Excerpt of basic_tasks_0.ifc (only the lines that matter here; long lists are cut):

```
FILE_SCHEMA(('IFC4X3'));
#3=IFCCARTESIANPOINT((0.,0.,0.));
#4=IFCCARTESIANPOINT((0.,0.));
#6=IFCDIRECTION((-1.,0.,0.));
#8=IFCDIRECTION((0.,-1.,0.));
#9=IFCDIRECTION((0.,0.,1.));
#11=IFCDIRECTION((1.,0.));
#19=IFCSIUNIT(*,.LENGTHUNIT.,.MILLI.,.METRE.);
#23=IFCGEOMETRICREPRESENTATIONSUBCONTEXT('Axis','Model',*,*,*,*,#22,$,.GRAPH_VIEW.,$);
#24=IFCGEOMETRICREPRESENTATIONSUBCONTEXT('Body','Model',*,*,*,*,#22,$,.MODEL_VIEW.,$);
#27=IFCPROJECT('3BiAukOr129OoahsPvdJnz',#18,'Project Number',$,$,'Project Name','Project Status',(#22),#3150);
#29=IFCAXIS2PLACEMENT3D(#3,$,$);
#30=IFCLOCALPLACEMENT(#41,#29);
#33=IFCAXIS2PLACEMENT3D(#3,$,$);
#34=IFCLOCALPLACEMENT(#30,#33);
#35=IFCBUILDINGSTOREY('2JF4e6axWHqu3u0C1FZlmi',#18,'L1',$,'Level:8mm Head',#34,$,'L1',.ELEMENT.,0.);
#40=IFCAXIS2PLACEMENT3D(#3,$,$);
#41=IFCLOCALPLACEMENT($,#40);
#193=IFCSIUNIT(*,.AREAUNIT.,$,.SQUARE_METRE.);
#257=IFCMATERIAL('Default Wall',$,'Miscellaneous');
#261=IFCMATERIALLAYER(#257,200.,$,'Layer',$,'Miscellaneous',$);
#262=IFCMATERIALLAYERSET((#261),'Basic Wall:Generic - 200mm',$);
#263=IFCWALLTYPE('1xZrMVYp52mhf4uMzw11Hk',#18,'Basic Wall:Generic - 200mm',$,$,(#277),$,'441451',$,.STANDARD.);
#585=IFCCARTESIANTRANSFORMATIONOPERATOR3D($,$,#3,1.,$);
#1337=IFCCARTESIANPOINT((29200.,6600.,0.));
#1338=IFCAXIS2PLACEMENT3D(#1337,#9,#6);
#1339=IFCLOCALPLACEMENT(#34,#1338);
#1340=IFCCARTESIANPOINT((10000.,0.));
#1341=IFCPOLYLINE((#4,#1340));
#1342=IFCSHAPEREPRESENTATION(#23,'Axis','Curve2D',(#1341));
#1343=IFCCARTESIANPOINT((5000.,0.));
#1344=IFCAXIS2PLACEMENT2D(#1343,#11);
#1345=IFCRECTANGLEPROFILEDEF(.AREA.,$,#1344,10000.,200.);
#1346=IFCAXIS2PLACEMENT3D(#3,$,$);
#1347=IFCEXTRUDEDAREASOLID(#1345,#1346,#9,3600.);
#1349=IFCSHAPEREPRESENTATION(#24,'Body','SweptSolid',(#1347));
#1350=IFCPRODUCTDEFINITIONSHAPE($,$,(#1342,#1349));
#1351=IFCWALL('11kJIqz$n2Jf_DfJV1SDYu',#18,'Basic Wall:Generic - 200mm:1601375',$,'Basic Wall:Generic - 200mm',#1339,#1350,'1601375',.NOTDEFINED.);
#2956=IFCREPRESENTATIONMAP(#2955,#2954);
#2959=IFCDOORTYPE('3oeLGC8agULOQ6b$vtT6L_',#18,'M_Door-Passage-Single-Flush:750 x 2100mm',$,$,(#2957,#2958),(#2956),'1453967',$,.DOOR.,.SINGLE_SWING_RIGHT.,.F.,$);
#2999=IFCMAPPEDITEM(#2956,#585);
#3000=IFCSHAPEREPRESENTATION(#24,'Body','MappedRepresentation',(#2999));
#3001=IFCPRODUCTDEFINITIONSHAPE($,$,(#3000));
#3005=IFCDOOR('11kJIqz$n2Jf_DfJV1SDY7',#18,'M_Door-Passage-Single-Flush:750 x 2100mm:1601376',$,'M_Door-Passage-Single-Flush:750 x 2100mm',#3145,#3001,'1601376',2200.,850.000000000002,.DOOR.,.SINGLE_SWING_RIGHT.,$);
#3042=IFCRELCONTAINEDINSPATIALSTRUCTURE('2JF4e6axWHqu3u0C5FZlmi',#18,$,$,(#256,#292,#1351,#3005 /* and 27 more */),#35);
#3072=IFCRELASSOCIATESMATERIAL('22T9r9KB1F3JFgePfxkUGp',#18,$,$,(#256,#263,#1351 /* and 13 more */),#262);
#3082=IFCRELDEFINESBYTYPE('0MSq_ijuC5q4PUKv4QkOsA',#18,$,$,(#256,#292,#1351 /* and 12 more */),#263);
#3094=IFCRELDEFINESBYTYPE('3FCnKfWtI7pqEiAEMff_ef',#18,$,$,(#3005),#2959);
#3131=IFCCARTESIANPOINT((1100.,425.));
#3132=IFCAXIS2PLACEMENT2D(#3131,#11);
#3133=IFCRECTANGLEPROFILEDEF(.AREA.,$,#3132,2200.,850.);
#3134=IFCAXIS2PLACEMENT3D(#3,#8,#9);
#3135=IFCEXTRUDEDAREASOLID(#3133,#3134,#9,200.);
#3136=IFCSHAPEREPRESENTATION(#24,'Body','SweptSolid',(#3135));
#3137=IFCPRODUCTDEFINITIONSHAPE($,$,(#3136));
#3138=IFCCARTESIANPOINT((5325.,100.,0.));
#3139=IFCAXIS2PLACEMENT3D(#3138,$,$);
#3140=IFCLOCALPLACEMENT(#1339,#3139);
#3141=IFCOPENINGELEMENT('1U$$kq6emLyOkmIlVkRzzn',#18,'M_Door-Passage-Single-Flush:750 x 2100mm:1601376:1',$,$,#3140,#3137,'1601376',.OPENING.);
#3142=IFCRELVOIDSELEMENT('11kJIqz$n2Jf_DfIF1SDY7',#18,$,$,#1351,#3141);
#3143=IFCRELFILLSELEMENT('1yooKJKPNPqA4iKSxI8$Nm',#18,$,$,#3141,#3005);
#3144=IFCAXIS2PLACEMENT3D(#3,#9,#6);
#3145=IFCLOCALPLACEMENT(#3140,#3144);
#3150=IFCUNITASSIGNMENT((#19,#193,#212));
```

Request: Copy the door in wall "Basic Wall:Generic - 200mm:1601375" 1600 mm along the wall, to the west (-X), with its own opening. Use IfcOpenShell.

```python
import ifcopenshell
import ifcopenshell.api.feature
import ifcopenshell.api.geometry
import ifcopenshell.api.root
import ifcopenshell.geom
import ifcopenshell.util.element
import ifcopenshell.util.placement
import ifcopenshell.util.shape
import ifcopenshell.util.unit

model = ifcopenshell.open("basic_tasks_0.ifc")
unit_scale = ifcopenshell.util.unit.calculate_unit_scale(model)
settings = ifcopenshell.geom.settings()


def volume(element):
    """Net volume in cubic metres, openings subtracted."""
    shape = ifcopenshell.geom.create_shape(settings, element)
    return ifcopenshell.util.shape.get_volume(shape.geometry)


def reuse_history(source, copy):
    """copy_class also copies each property set's owner history, people and application; keep the originals."""
    for rel in copy.IsDefinedBy:
        if rel.is_a("IfcRelDefinesByProperties") and (history := rel.RelatingPropertyDefinition.OwnerHistory):
            rel.RelatingPropertyDefinition.OwnerHistory = source.OwnerHistory
            ifcopenshell.util.element.remove_deep2(model, history)


door = model.by_guid("11kJIqz$n2Jf_DfJV1SDY7")
opening = door.FillsVoids[0].RelatingOpeningElement
wall = opening.VoidsElements[0].RelatingBuildingElement
before = volume(wall)
shift = ifcopenshell.util.placement.get_local_placement(wall.ObjectPlacement)[:3, 0] * 1.6 / unit_scale

# copy_class copies the void relationship, type, container and properties, but no geometry.
new_opening = ifcopenshell.api.root.copy_class(model, product=opening)
new_opening.Representation = ifcopenshell.util.element.copy_deep(
    model, opening.Representation, exclude=["IfcGeometricRepresentationContext", "IfcRepresentationMap"]
)
new_opening.Name = "M_Door-Passage-Single-Flush:750 x 2100mm"
new_opening.Tag = None
new_door = ifcopenshell.api.root.copy_class(model, product=door)
new_door.Representation = ifcopenshell.util.element.copy_deep(
    model, door.Representation, exclude=["IfcGeometricRepresentationContext", "IfcRepresentationMap"]
)
new_door.Name = "M_Door-Passage-Single-Flush:750 x 2100mm"
new_door.Tag = None
reuse_history(door, new_door)
ifcopenshell.api.feature.add_filling(model, opening=new_opening, element=new_door)

for old, new in ((opening, new_opening), (door, new_door)):
    matrix = ifcopenshell.util.placement.get_local_placement(old.ObjectPlacement)
    matrix[:3, 3] += shift
    ifcopenshell.api.geometry.edit_object_placement(model, product=new, matrix=matrix, is_si=False)

after = volume(wall)

print(f"wall volume {before:.3f} -> {after:.3f} m3")

model.write("basic_tasks_0_edited.ifc")
```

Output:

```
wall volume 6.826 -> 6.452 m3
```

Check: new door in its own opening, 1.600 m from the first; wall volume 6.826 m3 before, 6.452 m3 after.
